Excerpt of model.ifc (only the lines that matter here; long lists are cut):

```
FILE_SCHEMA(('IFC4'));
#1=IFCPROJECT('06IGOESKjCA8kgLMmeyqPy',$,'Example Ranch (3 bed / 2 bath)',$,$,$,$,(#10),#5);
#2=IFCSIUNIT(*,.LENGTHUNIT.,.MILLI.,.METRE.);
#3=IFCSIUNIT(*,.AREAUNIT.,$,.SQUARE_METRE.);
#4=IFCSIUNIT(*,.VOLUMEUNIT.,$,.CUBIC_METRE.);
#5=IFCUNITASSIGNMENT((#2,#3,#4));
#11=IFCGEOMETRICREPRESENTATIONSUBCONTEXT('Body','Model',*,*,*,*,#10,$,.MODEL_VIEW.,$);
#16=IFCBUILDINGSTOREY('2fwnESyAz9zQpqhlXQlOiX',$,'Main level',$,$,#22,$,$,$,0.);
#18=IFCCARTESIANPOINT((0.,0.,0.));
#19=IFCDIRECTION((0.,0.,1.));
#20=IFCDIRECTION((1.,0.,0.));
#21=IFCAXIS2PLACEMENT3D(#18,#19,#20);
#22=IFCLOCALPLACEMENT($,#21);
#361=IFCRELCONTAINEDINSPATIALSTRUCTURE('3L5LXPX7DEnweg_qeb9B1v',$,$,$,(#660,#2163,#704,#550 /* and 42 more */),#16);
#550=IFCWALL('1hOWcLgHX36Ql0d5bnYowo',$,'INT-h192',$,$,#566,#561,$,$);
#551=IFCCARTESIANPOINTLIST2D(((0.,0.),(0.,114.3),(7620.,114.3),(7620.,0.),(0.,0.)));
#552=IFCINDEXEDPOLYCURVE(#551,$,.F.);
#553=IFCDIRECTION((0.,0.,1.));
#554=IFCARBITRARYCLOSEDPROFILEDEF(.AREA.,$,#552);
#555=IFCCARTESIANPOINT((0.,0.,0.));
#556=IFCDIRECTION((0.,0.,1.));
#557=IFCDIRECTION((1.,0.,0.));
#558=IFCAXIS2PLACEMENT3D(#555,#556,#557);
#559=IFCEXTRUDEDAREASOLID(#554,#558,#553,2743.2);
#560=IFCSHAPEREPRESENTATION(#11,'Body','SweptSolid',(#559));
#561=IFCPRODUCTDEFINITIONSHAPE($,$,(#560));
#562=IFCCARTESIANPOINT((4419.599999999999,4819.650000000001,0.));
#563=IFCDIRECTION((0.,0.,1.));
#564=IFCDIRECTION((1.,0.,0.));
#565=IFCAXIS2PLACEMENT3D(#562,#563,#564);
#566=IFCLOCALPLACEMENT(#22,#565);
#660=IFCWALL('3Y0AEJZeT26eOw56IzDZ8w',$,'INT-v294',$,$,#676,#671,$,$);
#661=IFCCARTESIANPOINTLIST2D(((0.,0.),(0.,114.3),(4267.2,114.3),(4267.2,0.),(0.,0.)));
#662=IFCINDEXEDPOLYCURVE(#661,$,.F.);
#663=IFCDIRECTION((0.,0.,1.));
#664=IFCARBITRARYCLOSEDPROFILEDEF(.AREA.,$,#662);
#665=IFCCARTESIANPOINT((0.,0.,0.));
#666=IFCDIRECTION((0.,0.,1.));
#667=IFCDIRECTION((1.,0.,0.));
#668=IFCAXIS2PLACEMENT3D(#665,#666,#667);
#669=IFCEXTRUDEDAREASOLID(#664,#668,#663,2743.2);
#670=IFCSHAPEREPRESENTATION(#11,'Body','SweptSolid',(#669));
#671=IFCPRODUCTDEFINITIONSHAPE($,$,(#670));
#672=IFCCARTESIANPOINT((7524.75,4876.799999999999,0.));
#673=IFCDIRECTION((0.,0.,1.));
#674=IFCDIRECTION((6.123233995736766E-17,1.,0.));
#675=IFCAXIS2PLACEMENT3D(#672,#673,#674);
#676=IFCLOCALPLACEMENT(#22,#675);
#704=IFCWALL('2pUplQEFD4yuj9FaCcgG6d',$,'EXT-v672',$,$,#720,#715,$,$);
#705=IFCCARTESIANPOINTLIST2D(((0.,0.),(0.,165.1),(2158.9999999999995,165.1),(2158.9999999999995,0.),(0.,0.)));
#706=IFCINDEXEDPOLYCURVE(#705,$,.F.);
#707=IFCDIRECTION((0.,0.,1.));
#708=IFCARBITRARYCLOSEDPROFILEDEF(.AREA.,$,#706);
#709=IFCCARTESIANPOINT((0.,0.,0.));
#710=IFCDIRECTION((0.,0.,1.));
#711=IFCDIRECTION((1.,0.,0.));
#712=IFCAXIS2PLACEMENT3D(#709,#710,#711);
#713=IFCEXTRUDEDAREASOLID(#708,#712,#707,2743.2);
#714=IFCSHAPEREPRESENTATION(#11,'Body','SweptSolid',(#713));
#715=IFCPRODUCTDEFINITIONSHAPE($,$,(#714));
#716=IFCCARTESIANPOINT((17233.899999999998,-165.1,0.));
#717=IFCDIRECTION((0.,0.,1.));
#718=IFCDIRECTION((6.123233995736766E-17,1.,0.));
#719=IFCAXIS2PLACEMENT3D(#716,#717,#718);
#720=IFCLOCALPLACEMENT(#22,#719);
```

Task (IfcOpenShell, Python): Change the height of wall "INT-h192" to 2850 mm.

```python
import ifcopenshell
import ifcopenshell.geom
import ifcopenshell.util.representation
import ifcopenshell.util.shape

model = ifcopenshell.open("model.ifc")
settings = ifcopenshell.geom.settings()


def volume(element):
    """Net volume in cubic metres, openings subtracted."""
    shape = ifcopenshell.geom.create_shape(settings, element)
    return ifcopenshell.util.shape.get_volume(shape.geometry)


wall = model.by_guid("1hOWcLgHX36Ql0d5bnYowo")
before = volume(wall)

body = ifcopenshell.util.representation.get_representation(wall, "Model", "Body")
solid = body.Items[0]
old_height = solid.Depth
solid.Depth = 2850.0
after = volume(wall)

print(f"height {old_height:g} -> {solid.Depth:g}, volume {before:.3f} -> {after:.3f} m3")

model.write("model_updated.ifc")
```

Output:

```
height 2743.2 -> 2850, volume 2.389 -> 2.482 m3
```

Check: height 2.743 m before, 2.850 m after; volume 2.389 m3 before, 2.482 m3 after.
